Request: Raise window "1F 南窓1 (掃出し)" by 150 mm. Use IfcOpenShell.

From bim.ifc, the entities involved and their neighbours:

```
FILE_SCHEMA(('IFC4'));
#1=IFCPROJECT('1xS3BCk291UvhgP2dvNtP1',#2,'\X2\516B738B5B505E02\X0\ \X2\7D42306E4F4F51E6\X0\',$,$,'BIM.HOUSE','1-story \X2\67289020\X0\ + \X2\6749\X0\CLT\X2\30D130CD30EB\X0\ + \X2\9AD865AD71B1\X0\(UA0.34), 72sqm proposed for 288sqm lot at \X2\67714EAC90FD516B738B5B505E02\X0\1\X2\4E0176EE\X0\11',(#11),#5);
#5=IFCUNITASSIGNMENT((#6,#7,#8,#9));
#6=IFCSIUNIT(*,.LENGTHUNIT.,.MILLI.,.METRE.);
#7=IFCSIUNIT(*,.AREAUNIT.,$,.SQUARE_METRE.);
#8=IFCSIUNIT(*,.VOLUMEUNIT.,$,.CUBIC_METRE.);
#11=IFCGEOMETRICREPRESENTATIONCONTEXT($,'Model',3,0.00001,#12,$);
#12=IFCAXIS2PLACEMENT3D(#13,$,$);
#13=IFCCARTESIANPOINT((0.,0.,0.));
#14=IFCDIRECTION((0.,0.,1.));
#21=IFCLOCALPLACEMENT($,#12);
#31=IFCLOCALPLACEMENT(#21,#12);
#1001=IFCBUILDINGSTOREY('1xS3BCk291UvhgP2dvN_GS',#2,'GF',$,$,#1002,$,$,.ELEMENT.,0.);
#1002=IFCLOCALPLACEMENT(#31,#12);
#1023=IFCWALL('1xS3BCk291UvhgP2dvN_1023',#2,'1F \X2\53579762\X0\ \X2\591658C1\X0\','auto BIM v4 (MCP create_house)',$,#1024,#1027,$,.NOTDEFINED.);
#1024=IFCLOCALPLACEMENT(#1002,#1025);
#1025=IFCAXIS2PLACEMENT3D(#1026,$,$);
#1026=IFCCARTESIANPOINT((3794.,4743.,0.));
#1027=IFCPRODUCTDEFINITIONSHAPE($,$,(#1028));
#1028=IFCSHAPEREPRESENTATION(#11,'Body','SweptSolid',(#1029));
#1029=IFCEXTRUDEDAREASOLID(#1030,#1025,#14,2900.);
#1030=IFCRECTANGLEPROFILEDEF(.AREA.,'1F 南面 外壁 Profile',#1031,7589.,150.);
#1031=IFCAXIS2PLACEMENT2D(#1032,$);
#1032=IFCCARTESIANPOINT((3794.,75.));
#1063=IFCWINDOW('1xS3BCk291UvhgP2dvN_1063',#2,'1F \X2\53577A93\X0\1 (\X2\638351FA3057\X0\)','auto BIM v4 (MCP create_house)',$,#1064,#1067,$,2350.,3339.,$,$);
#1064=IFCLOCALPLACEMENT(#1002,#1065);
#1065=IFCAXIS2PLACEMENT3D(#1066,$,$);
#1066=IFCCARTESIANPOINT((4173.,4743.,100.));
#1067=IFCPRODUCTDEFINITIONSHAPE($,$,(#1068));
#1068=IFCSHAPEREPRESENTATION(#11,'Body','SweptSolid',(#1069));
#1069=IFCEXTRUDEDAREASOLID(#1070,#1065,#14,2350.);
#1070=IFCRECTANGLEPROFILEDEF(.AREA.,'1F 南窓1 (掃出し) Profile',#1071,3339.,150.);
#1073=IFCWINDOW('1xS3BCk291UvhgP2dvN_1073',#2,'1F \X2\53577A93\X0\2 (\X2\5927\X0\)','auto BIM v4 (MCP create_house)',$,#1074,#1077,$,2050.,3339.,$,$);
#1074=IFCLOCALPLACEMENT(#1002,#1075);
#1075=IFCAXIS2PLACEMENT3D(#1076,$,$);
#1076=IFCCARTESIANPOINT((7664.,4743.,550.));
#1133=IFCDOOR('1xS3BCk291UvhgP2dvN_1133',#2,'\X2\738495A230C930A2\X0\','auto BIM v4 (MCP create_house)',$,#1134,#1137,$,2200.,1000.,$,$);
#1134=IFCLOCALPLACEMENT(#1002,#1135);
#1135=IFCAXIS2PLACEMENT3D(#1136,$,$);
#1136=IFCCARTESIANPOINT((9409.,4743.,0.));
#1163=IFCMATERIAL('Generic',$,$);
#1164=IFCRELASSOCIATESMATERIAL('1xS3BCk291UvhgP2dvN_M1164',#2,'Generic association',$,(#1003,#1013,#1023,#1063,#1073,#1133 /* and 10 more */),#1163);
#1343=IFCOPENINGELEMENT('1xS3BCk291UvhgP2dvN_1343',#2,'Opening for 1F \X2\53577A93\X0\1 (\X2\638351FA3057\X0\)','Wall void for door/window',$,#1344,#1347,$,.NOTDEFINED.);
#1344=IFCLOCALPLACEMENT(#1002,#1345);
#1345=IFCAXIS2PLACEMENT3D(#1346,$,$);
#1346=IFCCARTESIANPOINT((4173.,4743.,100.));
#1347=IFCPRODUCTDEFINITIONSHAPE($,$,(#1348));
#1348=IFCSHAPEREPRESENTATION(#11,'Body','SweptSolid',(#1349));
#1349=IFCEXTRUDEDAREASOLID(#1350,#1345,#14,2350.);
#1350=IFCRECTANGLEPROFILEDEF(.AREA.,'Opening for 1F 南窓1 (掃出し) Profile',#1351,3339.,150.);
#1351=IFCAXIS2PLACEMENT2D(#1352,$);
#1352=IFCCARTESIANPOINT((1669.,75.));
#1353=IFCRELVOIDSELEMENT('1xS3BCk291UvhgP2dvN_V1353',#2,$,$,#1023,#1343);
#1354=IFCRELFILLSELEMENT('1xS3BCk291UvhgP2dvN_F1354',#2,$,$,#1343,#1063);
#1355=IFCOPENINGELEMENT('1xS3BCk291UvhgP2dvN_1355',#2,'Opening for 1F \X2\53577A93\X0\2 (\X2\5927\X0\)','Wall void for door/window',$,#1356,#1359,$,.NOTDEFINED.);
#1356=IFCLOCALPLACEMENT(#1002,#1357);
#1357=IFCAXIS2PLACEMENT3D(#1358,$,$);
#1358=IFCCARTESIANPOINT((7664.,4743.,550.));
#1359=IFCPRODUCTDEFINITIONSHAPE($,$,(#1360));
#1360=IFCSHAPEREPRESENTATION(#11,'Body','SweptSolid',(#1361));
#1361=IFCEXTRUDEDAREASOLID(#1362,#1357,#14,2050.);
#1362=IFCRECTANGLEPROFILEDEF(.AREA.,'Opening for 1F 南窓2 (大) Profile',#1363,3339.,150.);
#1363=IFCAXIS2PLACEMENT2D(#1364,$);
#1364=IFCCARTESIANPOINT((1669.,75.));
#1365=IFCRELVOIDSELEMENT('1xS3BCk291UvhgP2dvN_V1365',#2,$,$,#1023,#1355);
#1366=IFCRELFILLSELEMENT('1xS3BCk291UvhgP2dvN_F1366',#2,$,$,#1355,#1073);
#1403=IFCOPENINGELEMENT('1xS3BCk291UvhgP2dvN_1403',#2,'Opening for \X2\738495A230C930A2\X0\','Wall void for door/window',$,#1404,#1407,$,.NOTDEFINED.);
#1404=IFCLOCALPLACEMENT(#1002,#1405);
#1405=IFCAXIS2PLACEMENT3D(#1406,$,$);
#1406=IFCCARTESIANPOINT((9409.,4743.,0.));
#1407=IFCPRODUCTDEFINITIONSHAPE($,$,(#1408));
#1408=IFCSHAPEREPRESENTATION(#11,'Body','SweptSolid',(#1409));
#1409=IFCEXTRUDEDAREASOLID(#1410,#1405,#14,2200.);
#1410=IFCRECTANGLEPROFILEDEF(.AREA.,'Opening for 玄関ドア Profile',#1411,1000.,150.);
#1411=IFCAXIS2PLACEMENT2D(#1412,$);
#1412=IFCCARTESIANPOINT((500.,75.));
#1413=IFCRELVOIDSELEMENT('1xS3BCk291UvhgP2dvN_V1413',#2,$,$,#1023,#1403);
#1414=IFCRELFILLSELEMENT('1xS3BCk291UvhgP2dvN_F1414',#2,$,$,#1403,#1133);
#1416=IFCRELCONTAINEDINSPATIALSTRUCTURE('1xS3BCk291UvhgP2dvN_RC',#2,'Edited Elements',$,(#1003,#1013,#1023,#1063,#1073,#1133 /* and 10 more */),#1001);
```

```python
import numpy as np
import ifcopenshell
import ifcopenshell.api.geometry
import ifcopenshell.util.placement
import ifcopenshell.util.unit

model = ifcopenshell.open("bim.ifc")
unit_scale = ifcopenshell.util.unit.calculate_unit_scale(model)

window = model.by_guid("1xS3BCk291UvhgP2dvN_1063")
opening = window.FillsVoids[0].RelatingOpeningElement
dz = 0.15 / unit_scale

shift = np.array([0.0, 0.0, dz])
# The window is not placed relative to its opening, so move both.
for product in (opening, window):
    matrix = ifcopenshell.util.placement.get_local_placement(product.ObjectPlacement)
    matrix[:3, 3] += shift
    ifcopenshell.api.geometry.edit_object_placement(model, product=product, matrix=matrix, is_si=False)

print(f"moved by {dz * unit_scale:+.3f} m")

model.write("bim-out.ifc")
```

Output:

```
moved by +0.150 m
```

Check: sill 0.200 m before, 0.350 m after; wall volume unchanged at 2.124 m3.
